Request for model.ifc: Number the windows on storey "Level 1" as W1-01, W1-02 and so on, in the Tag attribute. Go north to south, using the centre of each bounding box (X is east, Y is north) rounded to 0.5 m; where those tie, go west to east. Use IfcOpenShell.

First a look at what the model holds.

```python
import ifcopenshell
import ifcopenshell.util.element
import ifcopenshell.util.placement

model = ifcopenshell.open("model.ifc")
print(model.schema)
storey = next(s for s in model.by_type("IfcBuildingStorey") if s.Name == "Level 1")
windows = [e for e in ifcopenshell.util.element.get_decomposition(storey) if e.is_a("IfcWindow")]
for e in sorted(windows, key=lambda e: e.id()):
    origin = ifcopenshell.util.placement.get_local_placement(e.ObjectPlacement)[:3, 3]
    print(e.id(), e.Tag, e.Name, origin.round(2) + 0.0, sep=" | ")
```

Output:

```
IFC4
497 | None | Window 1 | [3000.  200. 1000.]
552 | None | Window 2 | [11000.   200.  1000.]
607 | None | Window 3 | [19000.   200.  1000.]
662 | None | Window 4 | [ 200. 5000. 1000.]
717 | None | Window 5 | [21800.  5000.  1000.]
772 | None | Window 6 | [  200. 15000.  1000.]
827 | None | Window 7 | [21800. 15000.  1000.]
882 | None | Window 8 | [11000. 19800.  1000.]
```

```python
import ifcopenshell
import ifcopenshell.geom
import ifcopenshell.util.element
import ifcopenshell.util.shape

model = ifcopenshell.open("model.ifc")
settings = ifcopenshell.geom.settings()
settings.set("use-world-coords", True)


def centre(element):
    shape = ifcopenshell.geom.create_shape(settings, element)
    return ifcopenshell.util.shape.get_bbox_centroid(shape.geometry)


storey = next(s for s in model.by_type("IfcBuildingStorey") if s.Name == "Level 1")
windows = [e for e in ifcopenshell.util.element.get_decomposition(storey) if e.is_a("IfcWindow")]

# Insertion points can sit at a corner or the storey origin, so sort by the geometry (in metres).
centres = {e: centre(e) for e in windows}
windows.sort(key=lambda e: (-round(centres[e][1] / 0.5), centres[e][0]))

for i, e in enumerate(windows, start=1):
    number = f"W1-{i:02d}"
    e.Tag = number
    print(e.id(), number)

model.write("model_v2.ifc")
```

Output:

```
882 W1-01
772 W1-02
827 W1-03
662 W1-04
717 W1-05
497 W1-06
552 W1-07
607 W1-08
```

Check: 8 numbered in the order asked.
